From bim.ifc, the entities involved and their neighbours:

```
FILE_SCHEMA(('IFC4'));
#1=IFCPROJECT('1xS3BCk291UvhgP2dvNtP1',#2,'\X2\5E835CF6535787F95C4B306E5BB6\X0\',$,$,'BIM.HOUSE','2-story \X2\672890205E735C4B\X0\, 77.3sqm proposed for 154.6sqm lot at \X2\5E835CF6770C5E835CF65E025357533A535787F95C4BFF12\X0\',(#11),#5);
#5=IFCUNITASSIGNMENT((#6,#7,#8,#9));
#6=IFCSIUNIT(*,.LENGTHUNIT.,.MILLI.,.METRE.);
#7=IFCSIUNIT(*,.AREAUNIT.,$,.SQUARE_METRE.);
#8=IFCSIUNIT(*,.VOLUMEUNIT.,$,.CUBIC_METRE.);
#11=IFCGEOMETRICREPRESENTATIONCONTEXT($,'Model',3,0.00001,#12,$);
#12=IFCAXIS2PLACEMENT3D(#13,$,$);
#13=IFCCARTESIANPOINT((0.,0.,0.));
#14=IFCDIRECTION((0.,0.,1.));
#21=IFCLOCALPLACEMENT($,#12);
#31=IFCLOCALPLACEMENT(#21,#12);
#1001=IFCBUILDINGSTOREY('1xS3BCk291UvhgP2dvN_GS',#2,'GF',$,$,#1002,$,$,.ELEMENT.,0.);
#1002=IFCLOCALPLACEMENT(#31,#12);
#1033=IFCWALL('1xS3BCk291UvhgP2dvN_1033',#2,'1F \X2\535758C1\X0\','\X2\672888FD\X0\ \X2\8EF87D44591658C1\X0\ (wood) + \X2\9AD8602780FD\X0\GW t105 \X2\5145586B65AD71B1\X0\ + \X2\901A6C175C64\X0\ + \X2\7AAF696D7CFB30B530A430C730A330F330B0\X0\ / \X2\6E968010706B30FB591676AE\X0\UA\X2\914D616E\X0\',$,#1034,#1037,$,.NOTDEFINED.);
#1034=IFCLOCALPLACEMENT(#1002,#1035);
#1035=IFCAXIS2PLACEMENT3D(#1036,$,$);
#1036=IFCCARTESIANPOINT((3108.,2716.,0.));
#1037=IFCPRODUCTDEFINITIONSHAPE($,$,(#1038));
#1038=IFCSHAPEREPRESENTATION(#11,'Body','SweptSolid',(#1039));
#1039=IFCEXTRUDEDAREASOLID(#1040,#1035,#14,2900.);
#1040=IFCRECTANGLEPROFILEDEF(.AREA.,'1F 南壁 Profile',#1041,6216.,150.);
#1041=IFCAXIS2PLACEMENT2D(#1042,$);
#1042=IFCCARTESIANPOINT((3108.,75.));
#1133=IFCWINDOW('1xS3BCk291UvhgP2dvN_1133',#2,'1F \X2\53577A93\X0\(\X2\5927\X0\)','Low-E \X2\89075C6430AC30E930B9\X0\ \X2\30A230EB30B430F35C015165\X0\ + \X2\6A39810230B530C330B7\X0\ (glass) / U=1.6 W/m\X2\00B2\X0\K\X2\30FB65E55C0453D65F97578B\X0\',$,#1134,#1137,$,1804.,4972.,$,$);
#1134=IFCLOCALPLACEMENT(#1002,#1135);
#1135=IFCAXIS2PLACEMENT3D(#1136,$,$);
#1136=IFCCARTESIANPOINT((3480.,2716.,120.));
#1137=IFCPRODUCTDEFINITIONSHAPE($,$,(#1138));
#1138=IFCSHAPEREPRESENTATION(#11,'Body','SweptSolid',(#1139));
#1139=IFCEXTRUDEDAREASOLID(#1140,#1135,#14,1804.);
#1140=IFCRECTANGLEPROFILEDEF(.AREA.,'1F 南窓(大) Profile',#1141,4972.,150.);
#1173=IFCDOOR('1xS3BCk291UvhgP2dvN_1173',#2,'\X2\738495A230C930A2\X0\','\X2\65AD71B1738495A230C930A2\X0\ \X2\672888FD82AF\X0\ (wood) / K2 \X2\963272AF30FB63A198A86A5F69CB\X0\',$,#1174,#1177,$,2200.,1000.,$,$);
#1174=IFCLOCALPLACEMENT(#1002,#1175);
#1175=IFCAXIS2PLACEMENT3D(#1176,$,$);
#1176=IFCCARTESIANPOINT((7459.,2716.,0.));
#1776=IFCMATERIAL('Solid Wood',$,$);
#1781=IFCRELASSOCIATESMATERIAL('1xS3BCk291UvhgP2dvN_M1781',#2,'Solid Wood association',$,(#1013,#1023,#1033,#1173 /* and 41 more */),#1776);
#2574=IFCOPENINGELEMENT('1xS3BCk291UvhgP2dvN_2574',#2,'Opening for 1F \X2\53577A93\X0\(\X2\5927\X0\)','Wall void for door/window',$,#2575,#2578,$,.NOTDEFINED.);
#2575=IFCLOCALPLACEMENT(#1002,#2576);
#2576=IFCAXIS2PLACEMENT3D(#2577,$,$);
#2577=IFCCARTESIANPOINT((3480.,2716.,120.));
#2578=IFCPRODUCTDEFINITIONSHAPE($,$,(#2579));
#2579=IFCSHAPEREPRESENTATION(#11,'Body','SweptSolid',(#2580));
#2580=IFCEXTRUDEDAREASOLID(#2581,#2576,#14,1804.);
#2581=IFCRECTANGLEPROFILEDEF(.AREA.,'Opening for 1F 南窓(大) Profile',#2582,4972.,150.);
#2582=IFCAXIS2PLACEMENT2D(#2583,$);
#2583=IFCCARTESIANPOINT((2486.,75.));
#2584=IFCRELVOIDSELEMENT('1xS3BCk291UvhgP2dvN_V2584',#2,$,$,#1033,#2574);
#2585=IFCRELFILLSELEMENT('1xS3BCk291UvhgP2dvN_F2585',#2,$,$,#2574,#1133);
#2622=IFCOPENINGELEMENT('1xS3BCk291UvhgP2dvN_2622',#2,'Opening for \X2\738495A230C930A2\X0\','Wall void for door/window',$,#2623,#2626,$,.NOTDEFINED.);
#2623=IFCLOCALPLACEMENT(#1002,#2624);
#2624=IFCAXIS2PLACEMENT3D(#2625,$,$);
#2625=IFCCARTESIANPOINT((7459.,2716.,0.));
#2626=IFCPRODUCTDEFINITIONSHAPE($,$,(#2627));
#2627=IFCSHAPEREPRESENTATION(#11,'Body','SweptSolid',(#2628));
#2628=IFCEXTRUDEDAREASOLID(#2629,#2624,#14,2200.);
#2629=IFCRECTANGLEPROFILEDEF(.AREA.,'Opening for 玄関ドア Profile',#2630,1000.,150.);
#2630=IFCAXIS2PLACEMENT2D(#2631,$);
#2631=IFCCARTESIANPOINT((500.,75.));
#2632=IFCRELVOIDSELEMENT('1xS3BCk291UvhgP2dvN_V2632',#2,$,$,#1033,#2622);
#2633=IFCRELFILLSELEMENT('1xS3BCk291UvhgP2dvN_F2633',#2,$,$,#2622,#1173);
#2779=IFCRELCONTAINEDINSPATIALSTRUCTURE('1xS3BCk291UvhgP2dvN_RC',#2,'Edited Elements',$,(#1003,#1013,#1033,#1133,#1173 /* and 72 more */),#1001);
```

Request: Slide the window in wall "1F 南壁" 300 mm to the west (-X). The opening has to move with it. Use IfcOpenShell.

```python
import ifcopenshell
import ifcopenshell.api.geometry
import ifcopenshell.util.placement

model = ifcopenshell.open("bim.ifc")

window = model.by_guid("1xS3BCk291UvhgP2dvN_1133")
opening = window.FillsVoids[0].RelatingOpeningElement
wall = opening.VoidsElements[0].RelatingBuildingElement

wall_matrix = ifcopenshell.util.placement.get_local_placement(wall.ObjectPlacement)
shift = wall_matrix[:3, 0] * -300.0
before = ifcopenshell.util.placement.get_local_placement(window.ObjectPlacement)[:3, 3].copy()

# The window is not placed relative to its opening, so move both.
for product in (opening, window):
    matrix = ifcopenshell.util.placement.get_local_placement(product.ObjectPlacement)
    matrix[:3, 3] += shift
    ifcopenshell.api.geometry.edit_object_placement(model, product=product, matrix=matrix, is_si=False)

after = ifcopenshell.util.placement.get_local_placement(window.ObjectPlacement)[:3, 3]
print("window moved by", (after - before).round(3) + 0.0)

model.write("bim_v2.ifc")
```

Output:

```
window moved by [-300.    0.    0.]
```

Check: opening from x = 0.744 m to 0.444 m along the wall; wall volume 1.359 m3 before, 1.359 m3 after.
